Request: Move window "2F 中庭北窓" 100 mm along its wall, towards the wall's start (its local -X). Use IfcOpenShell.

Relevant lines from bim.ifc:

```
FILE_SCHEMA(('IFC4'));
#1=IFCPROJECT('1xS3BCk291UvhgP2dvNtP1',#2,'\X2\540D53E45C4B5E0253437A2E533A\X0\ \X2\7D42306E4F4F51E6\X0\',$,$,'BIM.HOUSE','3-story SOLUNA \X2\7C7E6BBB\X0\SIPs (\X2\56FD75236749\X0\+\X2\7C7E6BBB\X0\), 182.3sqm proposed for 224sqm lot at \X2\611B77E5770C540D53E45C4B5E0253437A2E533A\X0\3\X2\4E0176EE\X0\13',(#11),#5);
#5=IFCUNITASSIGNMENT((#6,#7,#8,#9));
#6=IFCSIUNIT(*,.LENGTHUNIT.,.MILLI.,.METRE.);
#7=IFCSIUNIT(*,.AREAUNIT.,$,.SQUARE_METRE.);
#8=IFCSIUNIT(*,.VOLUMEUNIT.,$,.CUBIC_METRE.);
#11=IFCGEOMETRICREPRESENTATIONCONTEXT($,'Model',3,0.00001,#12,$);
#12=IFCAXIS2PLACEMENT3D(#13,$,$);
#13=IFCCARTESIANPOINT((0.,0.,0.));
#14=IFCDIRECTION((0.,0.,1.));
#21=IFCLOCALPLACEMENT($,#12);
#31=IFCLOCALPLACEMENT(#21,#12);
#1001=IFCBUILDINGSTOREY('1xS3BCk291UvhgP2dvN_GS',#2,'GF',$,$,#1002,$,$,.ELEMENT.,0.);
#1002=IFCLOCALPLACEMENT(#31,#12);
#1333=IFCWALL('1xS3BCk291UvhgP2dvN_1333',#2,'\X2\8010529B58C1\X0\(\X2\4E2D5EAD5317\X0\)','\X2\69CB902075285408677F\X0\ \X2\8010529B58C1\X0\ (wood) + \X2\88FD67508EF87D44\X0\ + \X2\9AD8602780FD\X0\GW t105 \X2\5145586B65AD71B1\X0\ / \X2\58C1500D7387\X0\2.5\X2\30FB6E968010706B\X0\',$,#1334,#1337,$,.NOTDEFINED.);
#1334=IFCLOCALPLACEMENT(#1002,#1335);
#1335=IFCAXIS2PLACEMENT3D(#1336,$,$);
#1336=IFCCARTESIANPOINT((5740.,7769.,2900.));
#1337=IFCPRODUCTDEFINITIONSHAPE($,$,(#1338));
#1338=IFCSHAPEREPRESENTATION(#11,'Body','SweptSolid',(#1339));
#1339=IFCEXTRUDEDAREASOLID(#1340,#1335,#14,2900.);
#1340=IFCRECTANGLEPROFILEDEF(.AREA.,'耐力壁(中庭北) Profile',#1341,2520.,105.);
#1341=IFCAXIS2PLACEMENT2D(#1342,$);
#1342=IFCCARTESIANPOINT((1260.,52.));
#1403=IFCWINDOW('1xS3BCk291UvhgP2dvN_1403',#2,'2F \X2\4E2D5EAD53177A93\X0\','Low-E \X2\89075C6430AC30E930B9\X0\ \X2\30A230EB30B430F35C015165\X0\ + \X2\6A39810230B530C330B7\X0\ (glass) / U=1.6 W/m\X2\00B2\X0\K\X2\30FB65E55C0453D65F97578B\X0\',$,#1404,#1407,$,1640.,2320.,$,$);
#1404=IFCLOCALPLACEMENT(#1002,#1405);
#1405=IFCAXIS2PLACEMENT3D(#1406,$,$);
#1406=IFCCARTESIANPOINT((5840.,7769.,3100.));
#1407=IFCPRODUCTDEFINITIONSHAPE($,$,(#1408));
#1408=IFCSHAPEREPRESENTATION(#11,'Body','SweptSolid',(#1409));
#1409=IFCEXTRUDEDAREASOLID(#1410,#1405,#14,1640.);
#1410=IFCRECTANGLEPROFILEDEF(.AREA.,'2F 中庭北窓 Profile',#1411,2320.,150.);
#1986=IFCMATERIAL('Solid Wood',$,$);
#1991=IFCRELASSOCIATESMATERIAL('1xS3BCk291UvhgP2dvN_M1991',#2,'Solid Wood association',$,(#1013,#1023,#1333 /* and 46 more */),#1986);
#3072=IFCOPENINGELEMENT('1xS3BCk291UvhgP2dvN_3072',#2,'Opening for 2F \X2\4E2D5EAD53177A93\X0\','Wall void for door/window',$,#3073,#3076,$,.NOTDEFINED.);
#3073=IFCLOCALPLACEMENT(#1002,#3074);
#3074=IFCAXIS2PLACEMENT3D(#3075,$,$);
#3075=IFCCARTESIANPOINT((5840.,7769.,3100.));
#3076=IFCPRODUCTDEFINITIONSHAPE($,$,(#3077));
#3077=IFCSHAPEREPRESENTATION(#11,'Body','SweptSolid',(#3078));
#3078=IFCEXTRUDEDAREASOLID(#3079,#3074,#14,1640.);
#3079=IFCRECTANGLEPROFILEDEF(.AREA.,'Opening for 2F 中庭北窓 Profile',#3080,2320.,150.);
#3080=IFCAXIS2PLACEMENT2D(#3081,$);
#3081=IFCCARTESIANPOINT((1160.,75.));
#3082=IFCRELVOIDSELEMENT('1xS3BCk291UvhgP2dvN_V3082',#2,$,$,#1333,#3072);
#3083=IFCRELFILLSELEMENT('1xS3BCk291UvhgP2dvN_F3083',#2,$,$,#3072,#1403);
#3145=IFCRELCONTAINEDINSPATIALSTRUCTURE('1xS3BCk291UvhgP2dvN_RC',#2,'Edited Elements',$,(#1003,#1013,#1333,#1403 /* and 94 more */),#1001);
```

```python
import ifcopenshell
import ifcopenshell.api.geometry
import ifcopenshell.util.placement
import ifcopenshell.util.unit

model = ifcopenshell.open("bim.ifc")
unit_scale = ifcopenshell.util.unit.calculate_unit_scale(model)

window = model.by_id(1403)
opening = window.FillsVoids[0].RelatingOpeningElement
wall = opening.VoidsElements[0].RelatingBuildingElement

wall_matrix = ifcopenshell.util.placement.get_local_placement(wall.ObjectPlacement)
shift = wall_matrix[:3, 0] * -0.1 / unit_scale
before = ifcopenshell.util.placement.get_local_placement(window.ObjectPlacement)[:3, 3].copy()

# The window is not placed relative to its opening, so move both.
for product in (opening, window):
    matrix = ifcopenshell.util.placement.get_local_placement(product.ObjectPlacement)
    matrix[:3, 3] += shift
    ifcopenshell.api.geometry.edit_object_placement(model, product=product, matrix=matrix, is_si=False)

after = ifcopenshell.util.placement.get_local_placement(window.ObjectPlacement)[:3, 3]
print("window moved by", (after - before).round(3) + 0.0)

model.write("bim-out.ifc")
```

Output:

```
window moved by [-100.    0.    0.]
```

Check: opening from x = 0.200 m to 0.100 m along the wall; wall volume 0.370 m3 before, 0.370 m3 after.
